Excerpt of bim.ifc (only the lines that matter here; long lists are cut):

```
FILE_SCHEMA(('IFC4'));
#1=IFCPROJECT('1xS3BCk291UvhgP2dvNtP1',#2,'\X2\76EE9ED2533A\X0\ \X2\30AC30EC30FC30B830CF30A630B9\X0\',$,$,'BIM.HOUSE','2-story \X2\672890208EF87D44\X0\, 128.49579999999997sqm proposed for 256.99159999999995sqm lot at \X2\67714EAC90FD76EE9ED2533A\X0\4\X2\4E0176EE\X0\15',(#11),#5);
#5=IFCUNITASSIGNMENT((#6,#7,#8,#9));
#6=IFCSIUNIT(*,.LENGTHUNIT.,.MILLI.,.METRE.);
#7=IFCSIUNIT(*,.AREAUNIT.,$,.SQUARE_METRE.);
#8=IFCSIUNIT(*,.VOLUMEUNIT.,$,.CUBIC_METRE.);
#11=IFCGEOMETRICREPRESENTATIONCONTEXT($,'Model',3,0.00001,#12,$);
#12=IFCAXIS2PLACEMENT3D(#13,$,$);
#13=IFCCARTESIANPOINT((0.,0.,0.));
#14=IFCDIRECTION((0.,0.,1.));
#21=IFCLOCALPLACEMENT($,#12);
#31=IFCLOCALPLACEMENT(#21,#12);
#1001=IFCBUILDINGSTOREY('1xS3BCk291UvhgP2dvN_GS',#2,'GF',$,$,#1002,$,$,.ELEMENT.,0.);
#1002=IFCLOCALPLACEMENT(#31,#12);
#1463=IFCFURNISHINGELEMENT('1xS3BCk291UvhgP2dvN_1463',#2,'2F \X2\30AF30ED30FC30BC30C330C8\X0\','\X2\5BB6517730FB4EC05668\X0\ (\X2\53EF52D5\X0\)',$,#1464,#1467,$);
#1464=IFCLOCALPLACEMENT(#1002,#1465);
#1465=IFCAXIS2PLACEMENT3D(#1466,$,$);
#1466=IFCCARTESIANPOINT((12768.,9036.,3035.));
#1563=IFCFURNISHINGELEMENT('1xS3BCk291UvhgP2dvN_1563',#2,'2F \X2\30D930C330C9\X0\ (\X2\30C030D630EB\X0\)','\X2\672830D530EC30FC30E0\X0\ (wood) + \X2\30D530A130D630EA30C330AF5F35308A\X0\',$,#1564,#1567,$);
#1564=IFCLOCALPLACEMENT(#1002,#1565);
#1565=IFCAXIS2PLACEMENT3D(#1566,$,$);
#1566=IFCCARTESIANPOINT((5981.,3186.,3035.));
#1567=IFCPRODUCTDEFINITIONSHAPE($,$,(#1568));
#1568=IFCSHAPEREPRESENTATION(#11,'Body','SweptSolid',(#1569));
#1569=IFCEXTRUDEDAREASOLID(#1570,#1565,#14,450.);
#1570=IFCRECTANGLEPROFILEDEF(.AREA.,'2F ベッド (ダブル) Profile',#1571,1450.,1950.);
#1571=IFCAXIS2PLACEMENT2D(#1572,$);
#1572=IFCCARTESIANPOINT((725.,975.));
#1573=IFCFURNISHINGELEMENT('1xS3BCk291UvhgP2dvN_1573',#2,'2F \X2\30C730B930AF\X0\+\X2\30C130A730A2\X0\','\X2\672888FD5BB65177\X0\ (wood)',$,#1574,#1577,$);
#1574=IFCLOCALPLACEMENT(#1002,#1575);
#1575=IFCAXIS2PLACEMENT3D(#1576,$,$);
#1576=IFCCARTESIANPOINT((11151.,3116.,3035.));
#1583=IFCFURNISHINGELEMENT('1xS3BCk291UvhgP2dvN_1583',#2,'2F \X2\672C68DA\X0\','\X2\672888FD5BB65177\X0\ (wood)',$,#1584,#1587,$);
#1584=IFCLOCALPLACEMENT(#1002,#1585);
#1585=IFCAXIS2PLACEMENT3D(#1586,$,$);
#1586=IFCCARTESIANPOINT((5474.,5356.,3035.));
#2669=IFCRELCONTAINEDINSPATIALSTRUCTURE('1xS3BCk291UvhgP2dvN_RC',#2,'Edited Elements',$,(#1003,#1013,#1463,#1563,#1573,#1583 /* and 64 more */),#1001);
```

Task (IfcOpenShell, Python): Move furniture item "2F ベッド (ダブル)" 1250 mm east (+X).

```python
import ifcopenshell
import ifcopenshell.api.geometry
import ifcopenshell.util.placement

model = ifcopenshell.open("bim.ifc")

item = model.by_guid("1xS3BCk291UvhgP2dvN_1563")
matrix = ifcopenshell.util.placement.get_local_placement(item.ObjectPlacement)
matrix[0, 3] += 1250.0
ifcopenshell.api.geometry.edit_object_placement(model, product=item, matrix=matrix, is_si=False)

print(ifcopenshell.util.placement.get_local_placement(item.ObjectPlacement).round(3) + 0.0)

model.write("bim_rev.ifc")
```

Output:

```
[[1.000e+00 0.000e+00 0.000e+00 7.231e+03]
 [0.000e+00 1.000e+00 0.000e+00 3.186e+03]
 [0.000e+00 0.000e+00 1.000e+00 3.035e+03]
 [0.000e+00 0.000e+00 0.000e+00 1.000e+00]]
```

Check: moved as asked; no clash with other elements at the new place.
